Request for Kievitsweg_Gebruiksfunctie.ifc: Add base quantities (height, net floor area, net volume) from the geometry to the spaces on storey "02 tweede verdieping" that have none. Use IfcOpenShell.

First a look at what the model holds.

```python
import ifcopenshell
import ifcopenshell.util.element
import ifcopenshell.util.unit

model = ifcopenshell.open("Kievitsweg_Gebruiksfunctie.ifc")
print(model.schema)
for unit_type in ("LENGTHUNIT", "AREAUNIT", "VOLUMEUNIT"):
    print(unit_type, ifcopenshell.util.unit.calculate_unit_scale(model, unit_type))
storey = next(s for s in model.by_type("IfcBuildingStorey") if s.Name == "02 tweede verdieping")
spaces = [e for e in ifcopenshell.util.element.get_decomposition(storey) if e.is_a("IfcSpace")]
for e in sorted(spaces, key=lambda e: e.id()):
    print(e.id(), e.is_a(), e.Name, list(ifcopenshell.util.element.get_psets(e, qtos_only=True)), sep=" | ")
```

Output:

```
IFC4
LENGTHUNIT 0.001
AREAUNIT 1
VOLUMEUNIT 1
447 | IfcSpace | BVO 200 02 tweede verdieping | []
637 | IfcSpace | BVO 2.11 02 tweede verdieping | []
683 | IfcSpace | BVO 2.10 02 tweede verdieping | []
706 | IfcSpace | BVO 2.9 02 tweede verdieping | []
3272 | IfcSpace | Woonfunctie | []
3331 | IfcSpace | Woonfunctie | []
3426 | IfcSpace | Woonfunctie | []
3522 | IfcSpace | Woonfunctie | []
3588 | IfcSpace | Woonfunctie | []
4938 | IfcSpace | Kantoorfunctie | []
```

```python
import ifcopenshell
import ifcopenshell.api.pset
import ifcopenshell.geom
import ifcopenshell.util.element
import ifcopenshell.util.shape
import ifcopenshell.util.unit

model = ifcopenshell.open("Kievitsweg_Gebruiksfunctie.ifc")
unit_scale = ifcopenshell.util.unit.calculate_unit_scale(model)
area_scale = ifcopenshell.util.unit.calculate_unit_scale(model, "AREAUNIT")
volume_scale = ifcopenshell.util.unit.calculate_unit_scale(model, "VOLUMEUNIT")
settings = ifcopenshell.geom.settings()

storey = next(s for s in model.by_type("IfcBuildingStorey") if s.Name == "02 tweede verdieping")
spaces = [e for e in ifcopenshell.util.element.get_decomposition(storey) if e.is_a("IfcSpace")]

for e in sorted(spaces, key=lambda e: e.id()):
    if ifcopenshell.util.element.get_psets(e, qtos_only=True, should_inherit=False):
        continue
    # Geometry comes back in metres, in the element's own axes.
    shape = ifcopenshell.geom.create_shape(settings, e)
    values = {
        "Height": ifcopenshell.util.shape.get_z(shape.geometry) / unit_scale,
        "NetFloorArea": ifcopenshell.util.shape.get_footprint_area(shape.geometry) / area_scale,
        "NetVolume": ifcopenshell.util.shape.get_volume(shape.geometry) / volume_scale,
    }
    qto = ifcopenshell.api.pset.add_qto(model, product=e, name="Qto_SpaceBaseQuantities")
    ifcopenshell.api.pset.edit_qto(model, qto=qto, properties=values)
    print(e.id(), {k: round(v, 3) for k, v in values.items()})

model.write("Kievitsweg_Gebruiksfunctie_v2.ifc")
```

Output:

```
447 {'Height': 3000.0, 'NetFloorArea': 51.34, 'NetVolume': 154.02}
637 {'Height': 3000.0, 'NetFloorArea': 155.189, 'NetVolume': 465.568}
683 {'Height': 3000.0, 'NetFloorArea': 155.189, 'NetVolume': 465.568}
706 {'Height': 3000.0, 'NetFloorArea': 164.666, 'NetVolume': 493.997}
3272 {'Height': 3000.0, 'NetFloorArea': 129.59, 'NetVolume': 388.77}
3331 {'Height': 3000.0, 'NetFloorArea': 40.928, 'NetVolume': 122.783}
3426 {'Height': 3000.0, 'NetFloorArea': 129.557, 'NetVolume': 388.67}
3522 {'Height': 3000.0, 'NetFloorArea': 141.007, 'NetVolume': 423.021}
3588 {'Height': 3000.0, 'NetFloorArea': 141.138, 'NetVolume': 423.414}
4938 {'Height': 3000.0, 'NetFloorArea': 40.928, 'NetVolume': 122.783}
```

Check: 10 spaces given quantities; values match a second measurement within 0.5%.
